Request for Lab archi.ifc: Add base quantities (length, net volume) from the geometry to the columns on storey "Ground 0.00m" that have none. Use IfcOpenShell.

First a look at what the model holds.

```python
import ifcopenshell
import ifcopenshell.util.element
import ifcopenshell.util.unit

model = ifcopenshell.open("Lab archi.ifc")
print(model.schema)
for unit_type in ("LENGTHUNIT", "AREAUNIT", "VOLUMEUNIT"):
    print(unit_type, ifcopenshell.util.unit.calculate_unit_scale(model, unit_type))
storey = next(s for s in model.by_type("IfcBuildingStorey") if s.Name == "Ground 0.00m")
columns = [e for e in ifcopenshell.util.element.get_decomposition(storey) if e.is_a("IfcColumn")]
for e in sorted(columns, key=lambda e: e.id()):
    print(e.id(), e.is_a(), e.Name, list(ifcopenshell.util.element.get_psets(e, qtos_only=True)), sep=" | ")
```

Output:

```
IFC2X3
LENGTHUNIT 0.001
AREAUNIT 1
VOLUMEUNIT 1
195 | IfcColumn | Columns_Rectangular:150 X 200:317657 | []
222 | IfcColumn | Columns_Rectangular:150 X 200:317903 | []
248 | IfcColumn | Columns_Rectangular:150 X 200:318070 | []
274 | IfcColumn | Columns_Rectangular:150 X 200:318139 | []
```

```python
import ifcopenshell
import ifcopenshell.api.pset
import ifcopenshell.geom
import ifcopenshell.util.element
import ifcopenshell.util.shape
import ifcopenshell.util.unit

model = ifcopenshell.open("Lab archi.ifc")
unit_scale = ifcopenshell.util.unit.calculate_unit_scale(model)
volume_scale = ifcopenshell.util.unit.calculate_unit_scale(model, "VOLUMEUNIT")
settings = ifcopenshell.geom.settings()

storey = next(s for s in model.by_type("IfcBuildingStorey") if s.Name == "Ground 0.00m")
columns = [e for e in ifcopenshell.util.element.get_decomposition(storey) if e.is_a("IfcColumn")]

for e in sorted(columns, key=lambda e: e.id()):
    if ifcopenshell.util.element.get_psets(e, qtos_only=True, should_inherit=False):
        continue
    # Geometry comes back in metres, in the element's own axes.
    shape = ifcopenshell.geom.create_shape(settings, e)
    values = {
        "Length": ifcopenshell.util.shape.get_z(shape.geometry) / unit_scale,
        "NetVolume": ifcopenshell.util.shape.get_volume(shape.geometry) / volume_scale,
    }
    qto = ifcopenshell.api.pset.add_qto(model, product=e, name="BaseQuantities")
    ifcopenshell.api.pset.edit_qto(model, qto=qto, properties=values)
    print(e.id(), {k: round(v, 3) for k, v in values.items()})

model.write("Lab archi-out.ifc")
```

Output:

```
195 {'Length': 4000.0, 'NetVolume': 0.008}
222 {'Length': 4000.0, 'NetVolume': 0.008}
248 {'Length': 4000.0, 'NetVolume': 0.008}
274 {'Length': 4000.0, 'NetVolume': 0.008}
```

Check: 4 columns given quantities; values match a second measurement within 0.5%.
